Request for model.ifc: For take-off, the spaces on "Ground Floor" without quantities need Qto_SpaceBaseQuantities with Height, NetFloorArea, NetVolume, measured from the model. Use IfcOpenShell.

First a look at what the model holds.

```python
import ifcopenshell
import ifcopenshell.util.element
import ifcopenshell.util.unit

model = ifcopenshell.open("model.ifc")
print(model.schema)
for unit_type in ("LENGTHUNIT", "AREAUNIT", "VOLUMEUNIT"):
    print(unit_type, ifcopenshell.util.unit.calculate_unit_scale(model, unit_type))
storey = next(s for s in model.by_type("IfcBuildingStorey") if s.Name == "Ground Floor")
spaces = [e for e in ifcopenshell.util.element.get_decomposition(storey) if e.is_a("IfcSpace")]
for e in sorted(spaces, key=lambda e: e.id()):
    print(e.id(), e.is_a(), e.Name, list(ifcopenshell.util.element.get_psets(e, qtos_only=True)), sep=" | ")
```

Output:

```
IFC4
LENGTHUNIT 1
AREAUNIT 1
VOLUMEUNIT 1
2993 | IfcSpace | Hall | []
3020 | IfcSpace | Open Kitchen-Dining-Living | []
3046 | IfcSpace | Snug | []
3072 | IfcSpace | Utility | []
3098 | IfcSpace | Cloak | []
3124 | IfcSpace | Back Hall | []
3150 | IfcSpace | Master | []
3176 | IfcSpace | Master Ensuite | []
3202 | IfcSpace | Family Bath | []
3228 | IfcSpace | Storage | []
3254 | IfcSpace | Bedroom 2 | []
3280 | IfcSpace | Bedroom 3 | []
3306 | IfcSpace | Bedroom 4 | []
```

```python
import ifcopenshell
import ifcopenshell.api.pset
import ifcopenshell.geom
import ifcopenshell.util.element
import ifcopenshell.util.shape
import ifcopenshell.util.unit

model = ifcopenshell.open("model.ifc")
unit_scale = ifcopenshell.util.unit.calculate_unit_scale(model)
area_scale = ifcopenshell.util.unit.calculate_unit_scale(model, "AREAUNIT")
volume_scale = ifcopenshell.util.unit.calculate_unit_scale(model, "VOLUMEUNIT")
settings = ifcopenshell.geom.settings()

storey = next(s for s in model.by_type("IfcBuildingStorey") if s.Name == "Ground Floor")
spaces = [e for e in ifcopenshell.util.element.get_decomposition(storey) if e.is_a("IfcSpace")]

for e in sorted(spaces, key=lambda e: e.id()):
    if ifcopenshell.util.element.get_psets(e, qtos_only=True, should_inherit=False):
        continue
    # Geometry comes back in metres, in the element's own axes.
    shape = ifcopenshell.geom.create_shape(settings, e)
    values = {
        "Height": ifcopenshell.util.shape.get_z(shape.geometry) / unit_scale,
        "NetFloorArea": ifcopenshell.util.shape.get_footprint_area(shape.geometry) / area_scale,
        "NetVolume": ifcopenshell.util.shape.get_volume(shape.geometry) / volume_scale,
    }
    qto = ifcopenshell.api.pset.add_qto(model, product=e, name="Qto_SpaceBaseQuantities")
    ifcopenshell.api.pset.edit_qto(model, qto=qto, properties=values)
    print(e.id(), {k: round(v, 3) for k, v in values.items()})

model.write("model-out.ifc")
```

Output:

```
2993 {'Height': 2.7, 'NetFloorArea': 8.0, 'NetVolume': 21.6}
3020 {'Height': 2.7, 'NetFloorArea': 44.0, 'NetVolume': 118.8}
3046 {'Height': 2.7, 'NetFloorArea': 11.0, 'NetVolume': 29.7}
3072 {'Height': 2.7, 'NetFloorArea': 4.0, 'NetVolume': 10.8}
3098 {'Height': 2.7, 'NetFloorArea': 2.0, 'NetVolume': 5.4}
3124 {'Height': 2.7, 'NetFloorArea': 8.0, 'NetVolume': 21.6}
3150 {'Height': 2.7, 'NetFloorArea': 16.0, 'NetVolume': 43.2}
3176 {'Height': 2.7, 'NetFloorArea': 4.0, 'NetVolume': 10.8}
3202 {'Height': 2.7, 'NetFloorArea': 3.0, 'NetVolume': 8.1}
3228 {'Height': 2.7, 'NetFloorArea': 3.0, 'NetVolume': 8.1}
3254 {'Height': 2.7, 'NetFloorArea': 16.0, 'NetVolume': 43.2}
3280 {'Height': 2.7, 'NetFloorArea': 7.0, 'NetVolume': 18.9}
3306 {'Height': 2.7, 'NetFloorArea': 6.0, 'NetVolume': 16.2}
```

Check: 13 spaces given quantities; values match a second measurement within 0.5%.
